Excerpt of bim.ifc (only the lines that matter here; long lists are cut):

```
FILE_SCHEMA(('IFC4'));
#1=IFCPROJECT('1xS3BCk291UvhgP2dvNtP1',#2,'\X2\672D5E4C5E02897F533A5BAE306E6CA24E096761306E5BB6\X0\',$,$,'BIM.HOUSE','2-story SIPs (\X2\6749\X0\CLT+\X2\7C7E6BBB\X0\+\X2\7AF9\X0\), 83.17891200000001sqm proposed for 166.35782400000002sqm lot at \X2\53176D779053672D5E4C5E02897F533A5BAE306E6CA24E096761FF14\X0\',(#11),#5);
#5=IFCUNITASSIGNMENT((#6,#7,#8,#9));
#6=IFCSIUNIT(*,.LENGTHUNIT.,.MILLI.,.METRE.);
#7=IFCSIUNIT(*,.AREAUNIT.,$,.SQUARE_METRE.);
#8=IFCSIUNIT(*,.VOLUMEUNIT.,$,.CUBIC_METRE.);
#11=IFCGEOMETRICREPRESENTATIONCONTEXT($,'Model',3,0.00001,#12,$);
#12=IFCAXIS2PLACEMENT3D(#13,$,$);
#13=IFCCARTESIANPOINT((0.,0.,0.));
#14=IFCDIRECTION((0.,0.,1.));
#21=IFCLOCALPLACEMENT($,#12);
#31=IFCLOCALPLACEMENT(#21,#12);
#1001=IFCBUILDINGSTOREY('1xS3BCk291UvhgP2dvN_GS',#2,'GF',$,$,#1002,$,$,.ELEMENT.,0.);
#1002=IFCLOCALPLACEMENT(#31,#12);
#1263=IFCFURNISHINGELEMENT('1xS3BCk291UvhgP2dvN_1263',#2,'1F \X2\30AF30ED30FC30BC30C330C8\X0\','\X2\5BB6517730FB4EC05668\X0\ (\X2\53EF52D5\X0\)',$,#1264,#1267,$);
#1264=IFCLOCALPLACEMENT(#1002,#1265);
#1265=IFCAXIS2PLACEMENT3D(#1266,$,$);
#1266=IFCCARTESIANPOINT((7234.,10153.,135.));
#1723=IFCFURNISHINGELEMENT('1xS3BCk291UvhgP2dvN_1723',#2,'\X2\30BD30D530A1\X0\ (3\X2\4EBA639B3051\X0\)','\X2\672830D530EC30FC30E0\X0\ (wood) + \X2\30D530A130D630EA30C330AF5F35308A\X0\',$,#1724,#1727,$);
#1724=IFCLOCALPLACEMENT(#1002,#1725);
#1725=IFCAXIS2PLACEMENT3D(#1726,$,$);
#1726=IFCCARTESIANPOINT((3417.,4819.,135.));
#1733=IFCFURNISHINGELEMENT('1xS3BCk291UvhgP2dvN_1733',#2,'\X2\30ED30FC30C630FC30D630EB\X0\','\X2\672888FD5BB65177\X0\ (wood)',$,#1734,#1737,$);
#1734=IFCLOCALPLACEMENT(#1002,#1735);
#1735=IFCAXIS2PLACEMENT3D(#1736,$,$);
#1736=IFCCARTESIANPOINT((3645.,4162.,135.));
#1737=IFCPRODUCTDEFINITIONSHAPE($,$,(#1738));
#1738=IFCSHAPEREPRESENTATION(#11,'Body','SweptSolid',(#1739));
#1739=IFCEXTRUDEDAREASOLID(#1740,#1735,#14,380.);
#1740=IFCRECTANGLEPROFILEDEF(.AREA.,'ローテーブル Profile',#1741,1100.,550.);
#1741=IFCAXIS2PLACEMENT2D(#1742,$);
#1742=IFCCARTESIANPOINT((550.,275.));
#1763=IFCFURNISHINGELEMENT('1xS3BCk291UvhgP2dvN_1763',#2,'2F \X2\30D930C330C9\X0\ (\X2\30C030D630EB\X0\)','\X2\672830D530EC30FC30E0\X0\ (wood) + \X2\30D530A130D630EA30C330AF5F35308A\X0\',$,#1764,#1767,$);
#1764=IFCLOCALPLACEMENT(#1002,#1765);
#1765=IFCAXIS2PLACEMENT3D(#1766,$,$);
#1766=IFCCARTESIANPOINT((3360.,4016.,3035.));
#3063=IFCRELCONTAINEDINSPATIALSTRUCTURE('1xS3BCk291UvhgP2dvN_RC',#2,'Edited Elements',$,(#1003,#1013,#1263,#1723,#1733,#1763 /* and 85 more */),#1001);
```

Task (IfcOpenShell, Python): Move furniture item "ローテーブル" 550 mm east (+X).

```python
import ifcopenshell
import ifcopenshell.api.geometry
import ifcopenshell.util.placement
import ifcopenshell.util.unit

model = ifcopenshell.open("bim.ifc")
unit_scale = ifcopenshell.util.unit.calculate_unit_scale(model)

item = model.by_guid("1xS3BCk291UvhgP2dvN_1733")
matrix = ifcopenshell.util.placement.get_local_placement(item.ObjectPlacement)
matrix[0, 3] += 0.55 / unit_scale
ifcopenshell.api.geometry.edit_object_placement(model, product=item, matrix=matrix, is_si=False)

print(ifcopenshell.util.placement.get_local_placement(item.ObjectPlacement).round(3) + 0.0)

model.write("bim_updated.ifc")
```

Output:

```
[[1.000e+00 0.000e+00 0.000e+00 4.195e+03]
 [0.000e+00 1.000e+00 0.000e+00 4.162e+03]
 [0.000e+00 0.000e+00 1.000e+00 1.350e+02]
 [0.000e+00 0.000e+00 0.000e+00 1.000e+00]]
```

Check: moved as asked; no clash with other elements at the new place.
